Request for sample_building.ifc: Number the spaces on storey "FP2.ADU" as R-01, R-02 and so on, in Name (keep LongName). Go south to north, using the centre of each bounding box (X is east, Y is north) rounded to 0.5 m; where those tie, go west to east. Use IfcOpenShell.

First a look at what the model holds.

```python
import ifcopenshell
import ifcopenshell.util.element
import ifcopenshell.util.placement

model = ifcopenshell.open("sample_building.ifc")
print(model.schema)
storey = next(s for s in model.by_type("IfcBuildingStorey") if s.Name == "FP2.ADU")
spaces = [e for e in ifcopenshell.util.element.get_decomposition(storey) if e.is_a("IfcSpace")]
for e in sorted(spaces, key=lambda e: e.id()):
    origin = ifcopenshell.util.placement.get_local_placement(e.ObjectPlacement)[:3, 3]
    print(e.id(), e.Name, e.LongName, origin.round(2) + 0.0, sep=" | ")
```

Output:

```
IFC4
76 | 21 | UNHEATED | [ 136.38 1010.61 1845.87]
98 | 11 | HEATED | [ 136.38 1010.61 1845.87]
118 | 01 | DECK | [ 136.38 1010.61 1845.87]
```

```python
import ifcopenshell
import ifcopenshell.geom
import ifcopenshell.util.element
import ifcopenshell.util.shape

model = ifcopenshell.open("sample_building.ifc")
settings = ifcopenshell.geom.settings()
settings.set("use-world-coords", True)


def centre(element):
    shape = ifcopenshell.geom.create_shape(settings, element)
    return ifcopenshell.util.shape.get_bbox_centroid(shape.geometry)


storey = next(s for s in model.by_type("IfcBuildingStorey") if s.Name == "FP2.ADU")
spaces = [e for e in ifcopenshell.util.element.get_decomposition(storey) if e.is_a("IfcSpace")]

# Insertion points can sit at a corner or the storey origin, so sort by the geometry (in metres).
centres = {e: centre(e) for e in spaces}
spaces.sort(key=lambda e: (round(centres[e][1] / 0.5), centres[e][0]))

for i, e in enumerate(spaces, start=1):
    number = f"R-{i:02d}"
    e.Name = number
    print(e.id(), number)

model.write("sample_building_v2.ifc")
```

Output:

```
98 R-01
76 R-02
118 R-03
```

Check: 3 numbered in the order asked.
